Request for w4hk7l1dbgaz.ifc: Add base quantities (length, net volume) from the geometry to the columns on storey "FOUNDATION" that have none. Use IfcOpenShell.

First a look at what the model holds.

```python
import ifcopenshell
import ifcopenshell.util.element
import ifcopenshell.util.unit

model = ifcopenshell.open("w4hk7l1dbgaz.ifc")
print(model.schema)
for unit_type in ("LENGTHUNIT", "AREAUNIT", "VOLUMEUNIT"):
    print(unit_type, ifcopenshell.util.unit.calculate_unit_scale(model, unit_type))
storey = next(s for s in model.by_type("IfcBuildingStorey") if s.Name == "FOUNDATION")
columns = [e for e in ifcopenshell.util.element.get_decomposition(storey) if e.is_a("IfcColumn")]
for e in sorted(columns, key=lambda e: e.id()):
    print(e.id(), e.is_a(), e.Name, list(ifcopenshell.util.element.get_psets(e, qtos_only=True)), sep=" | ")
```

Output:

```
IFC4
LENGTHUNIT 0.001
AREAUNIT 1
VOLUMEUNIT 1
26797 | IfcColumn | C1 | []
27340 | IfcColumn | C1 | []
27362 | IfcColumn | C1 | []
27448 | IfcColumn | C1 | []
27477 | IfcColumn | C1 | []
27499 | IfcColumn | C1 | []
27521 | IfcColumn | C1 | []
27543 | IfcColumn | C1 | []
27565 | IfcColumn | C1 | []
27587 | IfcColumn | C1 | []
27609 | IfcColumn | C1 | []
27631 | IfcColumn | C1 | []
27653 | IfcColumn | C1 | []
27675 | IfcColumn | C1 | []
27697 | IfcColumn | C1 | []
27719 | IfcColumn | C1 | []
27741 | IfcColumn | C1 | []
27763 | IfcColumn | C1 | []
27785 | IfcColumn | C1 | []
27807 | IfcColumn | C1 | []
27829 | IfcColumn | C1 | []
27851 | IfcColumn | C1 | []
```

```python
import ifcopenshell
import ifcopenshell.api.pset
import ifcopenshell.geom
import ifcopenshell.util.element
import ifcopenshell.util.shape
import ifcopenshell.util.unit

model = ifcopenshell.open("w4hk7l1dbgaz.ifc")
unit_scale = ifcopenshell.util.unit.calculate_unit_scale(model)
volume_scale = ifcopenshell.util.unit.calculate_unit_scale(model, "VOLUMEUNIT")
settings = ifcopenshell.geom.settings()

storey = next(s for s in model.by_type("IfcBuildingStorey") if s.Name == "FOUNDATION")
columns = [e for e in ifcopenshell.util.element.get_decomposition(storey) if e.is_a("IfcColumn")]

for e in sorted(columns, key=lambda e: e.id()):
    if ifcopenshell.util.element.get_psets(e, qtos_only=True, should_inherit=False):
        continue
    # Geometry comes back in metres, in the element's own axes.
    shape = ifcopenshell.geom.create_shape(settings, e)
    values = {
        "Length": ifcopenshell.util.shape.get_z(shape.geometry) / unit_scale,
        "NetVolume": ifcopenshell.util.shape.get_volume(shape.geometry) / volume_scale,
    }
    qto = ifcopenshell.api.pset.add_qto(model, product=e, name="Qto_ColumnBaseQuantities")
    ifcopenshell.api.pset.edit_qto(model, qto=qto, properties=values)
    print(e.id(), {k: round(v, 3) for k, v in values.items()})

model.write("w4hk7l1dbgaz_edited.ifc")
```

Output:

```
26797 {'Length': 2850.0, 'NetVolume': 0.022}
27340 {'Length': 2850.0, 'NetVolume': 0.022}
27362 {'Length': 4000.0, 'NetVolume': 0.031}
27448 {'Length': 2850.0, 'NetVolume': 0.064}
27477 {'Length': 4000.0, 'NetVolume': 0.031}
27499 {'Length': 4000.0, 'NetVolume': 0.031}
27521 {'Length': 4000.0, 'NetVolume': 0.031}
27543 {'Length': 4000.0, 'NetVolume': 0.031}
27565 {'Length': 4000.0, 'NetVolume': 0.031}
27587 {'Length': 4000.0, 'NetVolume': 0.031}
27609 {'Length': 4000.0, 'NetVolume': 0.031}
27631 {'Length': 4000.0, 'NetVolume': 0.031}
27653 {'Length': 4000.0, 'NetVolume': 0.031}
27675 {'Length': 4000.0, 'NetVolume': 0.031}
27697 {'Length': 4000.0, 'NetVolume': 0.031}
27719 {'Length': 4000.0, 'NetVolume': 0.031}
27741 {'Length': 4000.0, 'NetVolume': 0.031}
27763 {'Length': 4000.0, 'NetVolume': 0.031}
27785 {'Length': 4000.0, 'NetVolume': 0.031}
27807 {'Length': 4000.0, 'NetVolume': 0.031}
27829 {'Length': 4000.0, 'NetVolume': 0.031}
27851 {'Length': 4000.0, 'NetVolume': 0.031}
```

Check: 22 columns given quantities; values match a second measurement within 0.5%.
